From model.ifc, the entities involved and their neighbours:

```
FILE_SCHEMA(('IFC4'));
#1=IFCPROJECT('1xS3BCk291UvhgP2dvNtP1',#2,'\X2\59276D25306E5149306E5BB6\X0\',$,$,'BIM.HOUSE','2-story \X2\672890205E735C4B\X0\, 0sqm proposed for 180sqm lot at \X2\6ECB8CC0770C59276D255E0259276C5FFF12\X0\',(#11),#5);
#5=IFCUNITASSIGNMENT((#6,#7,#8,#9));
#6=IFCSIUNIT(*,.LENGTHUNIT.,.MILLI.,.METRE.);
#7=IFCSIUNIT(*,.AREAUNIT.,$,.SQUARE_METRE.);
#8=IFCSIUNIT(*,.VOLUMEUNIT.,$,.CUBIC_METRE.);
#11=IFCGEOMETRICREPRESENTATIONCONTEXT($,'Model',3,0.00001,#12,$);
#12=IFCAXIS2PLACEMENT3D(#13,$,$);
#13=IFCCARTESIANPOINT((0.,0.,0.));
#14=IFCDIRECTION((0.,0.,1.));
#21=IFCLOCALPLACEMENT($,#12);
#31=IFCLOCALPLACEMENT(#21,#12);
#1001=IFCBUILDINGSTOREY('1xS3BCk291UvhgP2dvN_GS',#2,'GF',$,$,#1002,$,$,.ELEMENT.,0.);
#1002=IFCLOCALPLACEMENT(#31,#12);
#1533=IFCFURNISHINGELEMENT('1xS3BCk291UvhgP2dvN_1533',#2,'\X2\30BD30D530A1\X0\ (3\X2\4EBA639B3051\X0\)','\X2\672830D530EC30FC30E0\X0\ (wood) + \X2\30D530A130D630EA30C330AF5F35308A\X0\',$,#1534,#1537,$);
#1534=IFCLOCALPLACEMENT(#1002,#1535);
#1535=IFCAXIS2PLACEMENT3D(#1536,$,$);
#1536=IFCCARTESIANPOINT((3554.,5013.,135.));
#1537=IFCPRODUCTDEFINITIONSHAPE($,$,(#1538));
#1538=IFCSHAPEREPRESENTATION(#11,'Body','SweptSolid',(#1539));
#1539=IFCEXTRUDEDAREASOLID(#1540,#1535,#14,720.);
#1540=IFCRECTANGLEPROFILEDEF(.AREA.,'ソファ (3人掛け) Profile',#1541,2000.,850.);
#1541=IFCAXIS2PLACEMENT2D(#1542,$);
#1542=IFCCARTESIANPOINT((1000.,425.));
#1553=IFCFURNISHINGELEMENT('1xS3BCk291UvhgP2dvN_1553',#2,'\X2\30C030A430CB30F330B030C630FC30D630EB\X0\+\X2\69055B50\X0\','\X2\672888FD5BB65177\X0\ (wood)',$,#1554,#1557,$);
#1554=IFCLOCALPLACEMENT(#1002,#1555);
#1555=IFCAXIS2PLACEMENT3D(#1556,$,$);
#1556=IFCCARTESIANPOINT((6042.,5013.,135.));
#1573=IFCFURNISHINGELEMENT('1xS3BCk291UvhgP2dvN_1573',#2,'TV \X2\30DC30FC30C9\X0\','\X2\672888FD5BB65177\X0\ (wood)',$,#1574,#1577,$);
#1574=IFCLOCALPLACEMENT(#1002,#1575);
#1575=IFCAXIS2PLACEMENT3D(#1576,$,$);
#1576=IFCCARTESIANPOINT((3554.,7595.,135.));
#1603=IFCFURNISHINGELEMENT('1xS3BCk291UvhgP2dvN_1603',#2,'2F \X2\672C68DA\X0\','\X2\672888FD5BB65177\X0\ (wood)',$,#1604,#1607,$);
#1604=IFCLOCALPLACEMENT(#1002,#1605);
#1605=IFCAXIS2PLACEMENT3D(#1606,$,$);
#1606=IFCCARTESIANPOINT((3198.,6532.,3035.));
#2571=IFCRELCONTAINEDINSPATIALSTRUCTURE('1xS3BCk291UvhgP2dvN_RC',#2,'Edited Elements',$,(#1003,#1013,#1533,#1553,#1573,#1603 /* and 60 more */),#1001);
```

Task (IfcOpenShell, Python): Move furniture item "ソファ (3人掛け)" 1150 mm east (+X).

```python
import ifcopenshell
import ifcopenshell.api.geometry
import ifcopenshell.util.placement
import ifcopenshell.util.unit

model = ifcopenshell.open("model.ifc")
unit_scale = ifcopenshell.util.unit.calculate_unit_scale(model)

item = model.by_guid("1xS3BCk291UvhgP2dvN_1533")
matrix = ifcopenshell.util.placement.get_local_placement(item.ObjectPlacement)
matrix[0, 3] += 1.15 / unit_scale
ifcopenshell.api.geometry.edit_object_placement(model, product=item, matrix=matrix, is_si=False)

print(ifcopenshell.util.placement.get_local_placement(item.ObjectPlacement).round(3) + 0.0)

model.write("model_v2.ifc")
```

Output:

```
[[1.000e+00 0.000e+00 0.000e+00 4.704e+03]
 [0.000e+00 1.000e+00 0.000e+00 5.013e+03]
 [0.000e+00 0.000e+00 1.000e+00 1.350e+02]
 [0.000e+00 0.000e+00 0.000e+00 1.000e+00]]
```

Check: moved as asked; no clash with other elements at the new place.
